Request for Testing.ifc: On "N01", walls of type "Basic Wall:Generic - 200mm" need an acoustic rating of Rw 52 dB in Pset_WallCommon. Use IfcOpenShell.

First a look at what the model holds.

```python
import ifcopenshell
import ifcopenshell.util.element

model = ifcopenshell.open("Testing.ifc")
print(model.schema)
storey = next(s for s in model.by_type("IfcBuildingStorey") if s.Name == "N01")
walls = [e for e in ifcopenshell.util.element.get_decomposition(storey) if e.is_a("IfcWall")]
seen = {}
for e in walls:
    element_type = ifcopenshell.util.element.get_type(e)
    key = (element_type.Name if element_type != e and element_type else None, ifcopenshell.util.element.get_pset(e, "Pset_WallCommon", "AcousticRating"))
    seen[key] = seen.get(key, 0) + 1
for (name, value), count in sorted(seen.items(), key=str):
    print(count, "x", name, "|", value)
```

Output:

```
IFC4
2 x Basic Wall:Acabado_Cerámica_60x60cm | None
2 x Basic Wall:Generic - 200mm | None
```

```python
import ifcopenshell
import ifcopenshell.api.pset
import ifcopenshell.util.element

model = ifcopenshell.open("Testing.ifc")

storey = next(s for s in model.by_type("IfcBuildingStorey") if s.Name == "N01")
walls = [e for e in ifcopenshell.util.element.get_decomposition(storey) if e.is_a("IfcWall")]

count = 0
for e in walls:
    element_type = ifcopenshell.util.element.get_type(e)
    if element_type in (None, e) or element_type.Name != "Basic Wall:Generic - 200mm":
        continue
    # add_pset returns the element's existing set when there is one.
    pset = ifcopenshell.api.pset.add_pset(model, product=e, name="Pset_WallCommon")
    ifcopenshell.api.pset.edit_pset(model, pset=pset, properties={"AcousticRating": "Rw 52 dB"})
    count += 1

print(count, "walls updated")

model.write("Testing_rev.ifc")
```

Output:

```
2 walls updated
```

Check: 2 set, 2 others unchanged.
